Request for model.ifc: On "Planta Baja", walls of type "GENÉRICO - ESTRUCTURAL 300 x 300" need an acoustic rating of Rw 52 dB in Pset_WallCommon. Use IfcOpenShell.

First a look at what the model holds.

```python
import ifcopenshell
import ifcopenshell.util.element

model = ifcopenshell.open("model.ifc")
print(model.schema)
storey = next(s for s in model.by_type("IfcBuildingStorey") if s.Name == "Planta Baja")
walls = [e for e in ifcopenshell.util.element.get_decomposition(storey) if e.is_a("IfcWall")]
seen = {}
for e in walls:
    element_type = ifcopenshell.util.element.get_type(e)
    key = (element_type.Name if element_type != e and element_type else None, ifcopenshell.util.element.get_pset(e, "Pset_WallCommon", "AcousticRating"))
    seen[key] = seen.get(key, 0) + 1
for (name, value), count in sorted(seen.items(), key=str):
    print(count, "x", name, "|", value)
```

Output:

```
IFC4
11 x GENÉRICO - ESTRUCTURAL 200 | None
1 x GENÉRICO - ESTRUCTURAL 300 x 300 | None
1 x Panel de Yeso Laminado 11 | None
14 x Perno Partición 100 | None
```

```python
import ifcopenshell
import ifcopenshell.api.pset
import ifcopenshell.util.element

model = ifcopenshell.open("model.ifc")

storey = next(s for s in model.by_type("IfcBuildingStorey") if s.Name == "Planta Baja")
walls = [e for e in ifcopenshell.util.element.get_decomposition(storey) if e.is_a("IfcWall")]

count = 0
for e in walls:
    element_type = ifcopenshell.util.element.get_type(e)
    if element_type in (None, e) or element_type.Name != "GENÉRICO - ESTRUCTURAL 300 x 300":
        continue
    # add_pset returns the element's existing set when there is one.
    pset = ifcopenshell.api.pset.add_pset(model, product=e, name="Pset_WallCommon")
    ifcopenshell.api.pset.edit_pset(model, pset=pset, properties={"AcousticRating": "Rw 52 dB"})
    count += 1

print(count, "walls updated")

model.write("model-out.ifc")
```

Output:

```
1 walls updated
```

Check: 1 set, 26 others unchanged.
